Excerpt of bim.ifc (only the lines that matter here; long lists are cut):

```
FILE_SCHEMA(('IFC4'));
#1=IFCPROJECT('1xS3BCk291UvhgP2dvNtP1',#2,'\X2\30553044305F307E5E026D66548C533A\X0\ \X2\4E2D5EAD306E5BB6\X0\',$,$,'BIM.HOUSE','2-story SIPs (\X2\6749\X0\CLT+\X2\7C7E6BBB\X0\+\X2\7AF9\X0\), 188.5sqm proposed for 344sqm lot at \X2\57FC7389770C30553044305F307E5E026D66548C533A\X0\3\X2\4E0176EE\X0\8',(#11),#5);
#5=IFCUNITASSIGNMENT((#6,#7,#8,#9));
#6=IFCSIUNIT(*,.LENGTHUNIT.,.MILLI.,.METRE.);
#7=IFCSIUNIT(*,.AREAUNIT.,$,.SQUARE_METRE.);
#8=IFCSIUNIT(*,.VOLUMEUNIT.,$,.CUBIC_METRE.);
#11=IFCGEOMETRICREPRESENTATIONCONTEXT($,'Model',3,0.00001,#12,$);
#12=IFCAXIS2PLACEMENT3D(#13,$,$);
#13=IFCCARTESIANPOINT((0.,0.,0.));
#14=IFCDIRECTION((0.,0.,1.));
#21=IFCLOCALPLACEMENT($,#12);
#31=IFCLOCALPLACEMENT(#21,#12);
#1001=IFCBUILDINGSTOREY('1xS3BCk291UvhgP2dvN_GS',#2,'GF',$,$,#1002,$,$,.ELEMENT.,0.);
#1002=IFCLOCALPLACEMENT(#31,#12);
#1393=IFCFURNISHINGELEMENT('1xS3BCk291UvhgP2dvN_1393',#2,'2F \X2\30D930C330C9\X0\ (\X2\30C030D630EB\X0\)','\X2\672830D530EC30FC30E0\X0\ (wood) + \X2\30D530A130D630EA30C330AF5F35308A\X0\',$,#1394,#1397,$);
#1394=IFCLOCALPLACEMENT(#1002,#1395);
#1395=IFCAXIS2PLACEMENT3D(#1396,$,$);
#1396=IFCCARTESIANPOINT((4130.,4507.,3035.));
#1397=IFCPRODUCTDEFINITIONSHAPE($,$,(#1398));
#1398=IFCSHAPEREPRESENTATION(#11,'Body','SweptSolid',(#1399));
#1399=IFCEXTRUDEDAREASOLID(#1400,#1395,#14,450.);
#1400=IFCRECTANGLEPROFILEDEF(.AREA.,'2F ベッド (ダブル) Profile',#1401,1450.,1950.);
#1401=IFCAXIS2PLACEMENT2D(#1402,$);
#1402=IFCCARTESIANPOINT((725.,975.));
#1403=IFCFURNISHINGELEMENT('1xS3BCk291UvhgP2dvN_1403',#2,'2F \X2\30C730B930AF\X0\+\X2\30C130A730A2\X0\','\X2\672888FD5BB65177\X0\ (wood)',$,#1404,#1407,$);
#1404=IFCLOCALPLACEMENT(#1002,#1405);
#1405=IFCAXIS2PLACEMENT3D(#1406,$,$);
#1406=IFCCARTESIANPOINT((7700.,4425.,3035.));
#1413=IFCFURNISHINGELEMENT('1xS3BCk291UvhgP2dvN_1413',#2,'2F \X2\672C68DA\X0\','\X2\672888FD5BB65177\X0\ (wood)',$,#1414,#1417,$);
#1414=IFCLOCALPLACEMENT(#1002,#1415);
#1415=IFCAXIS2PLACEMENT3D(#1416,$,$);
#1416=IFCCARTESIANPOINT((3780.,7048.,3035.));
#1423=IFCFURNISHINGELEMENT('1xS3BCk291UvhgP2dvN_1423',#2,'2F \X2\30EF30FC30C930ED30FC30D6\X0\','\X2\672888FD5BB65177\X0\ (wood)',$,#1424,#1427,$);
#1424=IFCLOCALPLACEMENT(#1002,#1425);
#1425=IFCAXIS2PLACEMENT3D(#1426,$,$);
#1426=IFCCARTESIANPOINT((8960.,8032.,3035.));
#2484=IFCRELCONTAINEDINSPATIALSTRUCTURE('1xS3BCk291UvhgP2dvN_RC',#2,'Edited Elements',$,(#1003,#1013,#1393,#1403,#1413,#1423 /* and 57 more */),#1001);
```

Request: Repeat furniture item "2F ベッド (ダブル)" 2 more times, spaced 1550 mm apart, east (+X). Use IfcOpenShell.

```python
import numpy as np
import ifcopenshell
import ifcopenshell.api.geometry
import ifcopenshell.api.root
import ifcopenshell.util.element
import ifcopenshell.util.placement
import ifcopenshell.util.unit

model = ifcopenshell.open("bim.ifc")
unit_scale = ifcopenshell.util.unit.calculate_unit_scale(model)


def reuse_history(source, copy):
    """copy_class also copies each property set's owner history, people and application; keep the originals."""
    for rel in copy.IsDefinedBy:
        if rel.is_a("IfcRelDefinesByProperties") and (history := rel.RelatingPropertyDefinition.OwnerHistory):
            rel.RelatingPropertyDefinition.OwnerHistory = source.OwnerHistory
            ifcopenshell.util.element.remove_deep2(model, history)


source = model.by_guid("1xS3BCk291UvhgP2dvN_1393")
base = ifcopenshell.util.placement.get_local_placement(source.ObjectPlacement)
step = np.array([1.0, 0.0, 0.0]) * 1.55 / unit_scale

for i in range(1, 3):
    copy = ifcopenshell.api.root.copy_class(model, product=source)
    copy.Representation = ifcopenshell.util.element.copy_deep(
        model, source.Representation, exclude=["IfcGeometricRepresentationContext", "IfcRepresentationMap"]
    )
    reuse_history(source, copy)
    matrix = base.copy()
    matrix[:3, 3] += i * step
    print("added at", matrix[:3, 3].round(3) + 0.0)
    ifcopenshell.api.geometry.edit_object_placement(model, product=copy, matrix=matrix, is_si=False)

model.write("bim_v2.ifc")
```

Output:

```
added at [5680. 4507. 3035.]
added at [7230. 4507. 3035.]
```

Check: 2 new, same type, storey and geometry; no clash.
